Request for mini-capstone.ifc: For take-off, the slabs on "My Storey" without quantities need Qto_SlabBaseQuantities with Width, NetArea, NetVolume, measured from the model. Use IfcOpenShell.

First a look at what the model holds.

```python
import ifcopenshell
import ifcopenshell.util.element
import ifcopenshell.util.unit

model = ifcopenshell.open("mini-capstone.ifc")
print(model.schema)
for unit_type in ("LENGTHUNIT", "AREAUNIT", "VOLUMEUNIT"):
    print(unit_type, ifcopenshell.util.unit.calculate_unit_scale(model, unit_type))
storey = next(s for s in model.by_type("IfcBuildingStorey") if s.Name == "My Storey")
slabs = [e for e in ifcopenshell.util.element.get_decomposition(storey) if e.is_a("IfcSlab")]
for e in sorted(slabs, key=lambda e: e.id()):
    print(e.id(), e.is_a(), e.Name, list(ifcopenshell.util.element.get_psets(e, qtos_only=True)), sep=" | ")
```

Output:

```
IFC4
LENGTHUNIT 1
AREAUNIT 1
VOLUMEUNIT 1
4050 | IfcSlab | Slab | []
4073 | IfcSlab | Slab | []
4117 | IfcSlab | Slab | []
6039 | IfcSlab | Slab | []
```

```python
import ifcopenshell
import ifcopenshell.api.pset
import ifcopenshell.geom
import ifcopenshell.util.element
import ifcopenshell.util.shape
import ifcopenshell.util.unit

model = ifcopenshell.open("mini-capstone.ifc")
unit_scale = ifcopenshell.util.unit.calculate_unit_scale(model)
area_scale = ifcopenshell.util.unit.calculate_unit_scale(model, "AREAUNIT")
volume_scale = ifcopenshell.util.unit.calculate_unit_scale(model, "VOLUMEUNIT")
settings = ifcopenshell.geom.settings()

storey = next(s for s in model.by_type("IfcBuildingStorey") if s.Name == "My Storey")
slabs = [e for e in ifcopenshell.util.element.get_decomposition(storey) if e.is_a("IfcSlab")]

for e in sorted(slabs, key=lambda e: e.id()):
    if ifcopenshell.util.element.get_psets(e, qtos_only=True, should_inherit=False):
        continue
    # Geometry comes back in metres, in the element's own axes.
    shape = ifcopenshell.geom.create_shape(settings, e)
    values = {
        "Width": ifcopenshell.util.shape.get_z(shape.geometry) / unit_scale,
        "NetArea": ifcopenshell.util.shape.get_footprint_area(shape.geometry) / area_scale,
        "NetVolume": ifcopenshell.util.shape.get_volume(shape.geometry) / volume_scale,
    }
    qto = ifcopenshell.api.pset.add_qto(model, product=e, name="Qto_SlabBaseQuantities")
    ifcopenshell.api.pset.edit_qto(model, qto=qto, properties=values)
    print(e.id(), {k: round(v, 3) for k, v in values.items()})

model.write("mini-capstone-out.ifc")
```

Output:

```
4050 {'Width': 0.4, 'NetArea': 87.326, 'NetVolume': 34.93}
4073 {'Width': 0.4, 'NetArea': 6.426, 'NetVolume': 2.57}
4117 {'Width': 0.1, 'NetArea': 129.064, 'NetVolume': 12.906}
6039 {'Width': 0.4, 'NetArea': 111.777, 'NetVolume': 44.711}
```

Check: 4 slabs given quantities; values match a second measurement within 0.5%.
